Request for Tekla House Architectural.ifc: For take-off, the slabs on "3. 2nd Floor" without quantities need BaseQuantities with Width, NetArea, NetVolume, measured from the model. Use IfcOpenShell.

First a look at what the model holds.

```python
import ifcopenshell
import ifcopenshell.util.element
import ifcopenshell.util.unit

model = ifcopenshell.open("Tekla House Architectural.ifc")
print(model.schema)
for unit_type in ("LENGTHUNIT", "AREAUNIT", "VOLUMEUNIT"):
    print(unit_type, ifcopenshell.util.unit.calculate_unit_scale(model, unit_type))
storey = next(s for s in model.by_type("IfcBuildingStorey") if s.Name == "3. 2nd Floor")
slabs = [e for e in ifcopenshell.util.element.get_decomposition(storey) if e.is_a("IfcSlab")]
for e in sorted(slabs, key=lambda e: e.id()):
    print(e.id(), e.is_a(), e.Name, list(ifcopenshell.util.element.get_psets(e, qtos_only=True)), sep=" | ")
```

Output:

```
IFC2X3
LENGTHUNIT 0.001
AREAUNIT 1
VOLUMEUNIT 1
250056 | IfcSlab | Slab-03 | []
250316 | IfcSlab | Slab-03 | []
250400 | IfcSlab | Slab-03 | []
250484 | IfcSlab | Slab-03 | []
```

```python
import ifcopenshell
import ifcopenshell.api.pset
import ifcopenshell.geom
import ifcopenshell.util.element
import ifcopenshell.util.shape
import ifcopenshell.util.unit

model = ifcopenshell.open("Tekla House Architectural.ifc")
unit_scale = ifcopenshell.util.unit.calculate_unit_scale(model)
area_scale = ifcopenshell.util.unit.calculate_unit_scale(model, "AREAUNIT")
volume_scale = ifcopenshell.util.unit.calculate_unit_scale(model, "VOLUMEUNIT")
settings = ifcopenshell.geom.settings()

storey = next(s for s in model.by_type("IfcBuildingStorey") if s.Name == "3. 2nd Floor")
slabs = [e for e in ifcopenshell.util.element.get_decomposition(storey) if e.is_a("IfcSlab")]

for e in sorted(slabs, key=lambda e: e.id()):
    if ifcopenshell.util.element.get_psets(e, qtos_only=True, should_inherit=False):
        continue
    # Geometry comes back in metres, in the element's own axes.
    shape = ifcopenshell.geom.create_shape(settings, e)
    values = {
        "Width": ifcopenshell.util.shape.get_z(shape.geometry) / unit_scale,
        "NetArea": ifcopenshell.util.shape.get_footprint_area(shape.geometry) / area_scale,
        "NetVolume": ifcopenshell.util.shape.get_volume(shape.geometry) / volume_scale,
    }
    qto = ifcopenshell.api.pset.add_qto(model, product=e, name="BaseQuantities")
    ifcopenshell.api.pset.edit_qto(model, qto=qto, properties=values)
    print(e.id(), {k: round(v, 3) for k, v in values.items()})

model.write("Tekla House Architectural_rev.ifc")
```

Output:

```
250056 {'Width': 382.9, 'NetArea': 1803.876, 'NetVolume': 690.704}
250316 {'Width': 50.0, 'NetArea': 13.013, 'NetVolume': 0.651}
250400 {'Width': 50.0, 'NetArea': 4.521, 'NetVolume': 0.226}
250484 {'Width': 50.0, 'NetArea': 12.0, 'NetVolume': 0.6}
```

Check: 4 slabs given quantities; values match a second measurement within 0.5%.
